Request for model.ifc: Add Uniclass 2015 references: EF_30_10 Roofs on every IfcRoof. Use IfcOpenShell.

First a look at what the model holds.

```python
import ifcopenshell

model = ifcopenshell.open("model.ifc")
print(model.schema)
print("classifications:", [c.Name for c in model.by_type("IfcClassification")])
for ifc_class in ("IfcDoor", "IfcRoof", "IfcStair", "IfcWall", "IfcWindow"):
    print(ifc_class, len(model.by_type(ifc_class)))
```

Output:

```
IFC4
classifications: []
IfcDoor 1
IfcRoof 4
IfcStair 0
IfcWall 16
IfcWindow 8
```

```python
import ifcopenshell
import ifcopenshell.api.classification

model = ifcopenshell.open("model.ifc")

system = ifcopenshell.api.classification.add_classification(model, classification="Uniclass 2015")

codes = {
    "IfcRoof": ("EF_30_10", "Roofs"),
}
for ifc_class, (code, name) in codes.items():
    products = model.by_type(ifc_class)
    ifcopenshell.api.classification.add_reference(
        model, products=products, classification=system, identification=code, name=name
    )
    print(code, len(products))

model.write("model_v2.ifc")
```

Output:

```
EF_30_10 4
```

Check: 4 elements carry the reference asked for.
